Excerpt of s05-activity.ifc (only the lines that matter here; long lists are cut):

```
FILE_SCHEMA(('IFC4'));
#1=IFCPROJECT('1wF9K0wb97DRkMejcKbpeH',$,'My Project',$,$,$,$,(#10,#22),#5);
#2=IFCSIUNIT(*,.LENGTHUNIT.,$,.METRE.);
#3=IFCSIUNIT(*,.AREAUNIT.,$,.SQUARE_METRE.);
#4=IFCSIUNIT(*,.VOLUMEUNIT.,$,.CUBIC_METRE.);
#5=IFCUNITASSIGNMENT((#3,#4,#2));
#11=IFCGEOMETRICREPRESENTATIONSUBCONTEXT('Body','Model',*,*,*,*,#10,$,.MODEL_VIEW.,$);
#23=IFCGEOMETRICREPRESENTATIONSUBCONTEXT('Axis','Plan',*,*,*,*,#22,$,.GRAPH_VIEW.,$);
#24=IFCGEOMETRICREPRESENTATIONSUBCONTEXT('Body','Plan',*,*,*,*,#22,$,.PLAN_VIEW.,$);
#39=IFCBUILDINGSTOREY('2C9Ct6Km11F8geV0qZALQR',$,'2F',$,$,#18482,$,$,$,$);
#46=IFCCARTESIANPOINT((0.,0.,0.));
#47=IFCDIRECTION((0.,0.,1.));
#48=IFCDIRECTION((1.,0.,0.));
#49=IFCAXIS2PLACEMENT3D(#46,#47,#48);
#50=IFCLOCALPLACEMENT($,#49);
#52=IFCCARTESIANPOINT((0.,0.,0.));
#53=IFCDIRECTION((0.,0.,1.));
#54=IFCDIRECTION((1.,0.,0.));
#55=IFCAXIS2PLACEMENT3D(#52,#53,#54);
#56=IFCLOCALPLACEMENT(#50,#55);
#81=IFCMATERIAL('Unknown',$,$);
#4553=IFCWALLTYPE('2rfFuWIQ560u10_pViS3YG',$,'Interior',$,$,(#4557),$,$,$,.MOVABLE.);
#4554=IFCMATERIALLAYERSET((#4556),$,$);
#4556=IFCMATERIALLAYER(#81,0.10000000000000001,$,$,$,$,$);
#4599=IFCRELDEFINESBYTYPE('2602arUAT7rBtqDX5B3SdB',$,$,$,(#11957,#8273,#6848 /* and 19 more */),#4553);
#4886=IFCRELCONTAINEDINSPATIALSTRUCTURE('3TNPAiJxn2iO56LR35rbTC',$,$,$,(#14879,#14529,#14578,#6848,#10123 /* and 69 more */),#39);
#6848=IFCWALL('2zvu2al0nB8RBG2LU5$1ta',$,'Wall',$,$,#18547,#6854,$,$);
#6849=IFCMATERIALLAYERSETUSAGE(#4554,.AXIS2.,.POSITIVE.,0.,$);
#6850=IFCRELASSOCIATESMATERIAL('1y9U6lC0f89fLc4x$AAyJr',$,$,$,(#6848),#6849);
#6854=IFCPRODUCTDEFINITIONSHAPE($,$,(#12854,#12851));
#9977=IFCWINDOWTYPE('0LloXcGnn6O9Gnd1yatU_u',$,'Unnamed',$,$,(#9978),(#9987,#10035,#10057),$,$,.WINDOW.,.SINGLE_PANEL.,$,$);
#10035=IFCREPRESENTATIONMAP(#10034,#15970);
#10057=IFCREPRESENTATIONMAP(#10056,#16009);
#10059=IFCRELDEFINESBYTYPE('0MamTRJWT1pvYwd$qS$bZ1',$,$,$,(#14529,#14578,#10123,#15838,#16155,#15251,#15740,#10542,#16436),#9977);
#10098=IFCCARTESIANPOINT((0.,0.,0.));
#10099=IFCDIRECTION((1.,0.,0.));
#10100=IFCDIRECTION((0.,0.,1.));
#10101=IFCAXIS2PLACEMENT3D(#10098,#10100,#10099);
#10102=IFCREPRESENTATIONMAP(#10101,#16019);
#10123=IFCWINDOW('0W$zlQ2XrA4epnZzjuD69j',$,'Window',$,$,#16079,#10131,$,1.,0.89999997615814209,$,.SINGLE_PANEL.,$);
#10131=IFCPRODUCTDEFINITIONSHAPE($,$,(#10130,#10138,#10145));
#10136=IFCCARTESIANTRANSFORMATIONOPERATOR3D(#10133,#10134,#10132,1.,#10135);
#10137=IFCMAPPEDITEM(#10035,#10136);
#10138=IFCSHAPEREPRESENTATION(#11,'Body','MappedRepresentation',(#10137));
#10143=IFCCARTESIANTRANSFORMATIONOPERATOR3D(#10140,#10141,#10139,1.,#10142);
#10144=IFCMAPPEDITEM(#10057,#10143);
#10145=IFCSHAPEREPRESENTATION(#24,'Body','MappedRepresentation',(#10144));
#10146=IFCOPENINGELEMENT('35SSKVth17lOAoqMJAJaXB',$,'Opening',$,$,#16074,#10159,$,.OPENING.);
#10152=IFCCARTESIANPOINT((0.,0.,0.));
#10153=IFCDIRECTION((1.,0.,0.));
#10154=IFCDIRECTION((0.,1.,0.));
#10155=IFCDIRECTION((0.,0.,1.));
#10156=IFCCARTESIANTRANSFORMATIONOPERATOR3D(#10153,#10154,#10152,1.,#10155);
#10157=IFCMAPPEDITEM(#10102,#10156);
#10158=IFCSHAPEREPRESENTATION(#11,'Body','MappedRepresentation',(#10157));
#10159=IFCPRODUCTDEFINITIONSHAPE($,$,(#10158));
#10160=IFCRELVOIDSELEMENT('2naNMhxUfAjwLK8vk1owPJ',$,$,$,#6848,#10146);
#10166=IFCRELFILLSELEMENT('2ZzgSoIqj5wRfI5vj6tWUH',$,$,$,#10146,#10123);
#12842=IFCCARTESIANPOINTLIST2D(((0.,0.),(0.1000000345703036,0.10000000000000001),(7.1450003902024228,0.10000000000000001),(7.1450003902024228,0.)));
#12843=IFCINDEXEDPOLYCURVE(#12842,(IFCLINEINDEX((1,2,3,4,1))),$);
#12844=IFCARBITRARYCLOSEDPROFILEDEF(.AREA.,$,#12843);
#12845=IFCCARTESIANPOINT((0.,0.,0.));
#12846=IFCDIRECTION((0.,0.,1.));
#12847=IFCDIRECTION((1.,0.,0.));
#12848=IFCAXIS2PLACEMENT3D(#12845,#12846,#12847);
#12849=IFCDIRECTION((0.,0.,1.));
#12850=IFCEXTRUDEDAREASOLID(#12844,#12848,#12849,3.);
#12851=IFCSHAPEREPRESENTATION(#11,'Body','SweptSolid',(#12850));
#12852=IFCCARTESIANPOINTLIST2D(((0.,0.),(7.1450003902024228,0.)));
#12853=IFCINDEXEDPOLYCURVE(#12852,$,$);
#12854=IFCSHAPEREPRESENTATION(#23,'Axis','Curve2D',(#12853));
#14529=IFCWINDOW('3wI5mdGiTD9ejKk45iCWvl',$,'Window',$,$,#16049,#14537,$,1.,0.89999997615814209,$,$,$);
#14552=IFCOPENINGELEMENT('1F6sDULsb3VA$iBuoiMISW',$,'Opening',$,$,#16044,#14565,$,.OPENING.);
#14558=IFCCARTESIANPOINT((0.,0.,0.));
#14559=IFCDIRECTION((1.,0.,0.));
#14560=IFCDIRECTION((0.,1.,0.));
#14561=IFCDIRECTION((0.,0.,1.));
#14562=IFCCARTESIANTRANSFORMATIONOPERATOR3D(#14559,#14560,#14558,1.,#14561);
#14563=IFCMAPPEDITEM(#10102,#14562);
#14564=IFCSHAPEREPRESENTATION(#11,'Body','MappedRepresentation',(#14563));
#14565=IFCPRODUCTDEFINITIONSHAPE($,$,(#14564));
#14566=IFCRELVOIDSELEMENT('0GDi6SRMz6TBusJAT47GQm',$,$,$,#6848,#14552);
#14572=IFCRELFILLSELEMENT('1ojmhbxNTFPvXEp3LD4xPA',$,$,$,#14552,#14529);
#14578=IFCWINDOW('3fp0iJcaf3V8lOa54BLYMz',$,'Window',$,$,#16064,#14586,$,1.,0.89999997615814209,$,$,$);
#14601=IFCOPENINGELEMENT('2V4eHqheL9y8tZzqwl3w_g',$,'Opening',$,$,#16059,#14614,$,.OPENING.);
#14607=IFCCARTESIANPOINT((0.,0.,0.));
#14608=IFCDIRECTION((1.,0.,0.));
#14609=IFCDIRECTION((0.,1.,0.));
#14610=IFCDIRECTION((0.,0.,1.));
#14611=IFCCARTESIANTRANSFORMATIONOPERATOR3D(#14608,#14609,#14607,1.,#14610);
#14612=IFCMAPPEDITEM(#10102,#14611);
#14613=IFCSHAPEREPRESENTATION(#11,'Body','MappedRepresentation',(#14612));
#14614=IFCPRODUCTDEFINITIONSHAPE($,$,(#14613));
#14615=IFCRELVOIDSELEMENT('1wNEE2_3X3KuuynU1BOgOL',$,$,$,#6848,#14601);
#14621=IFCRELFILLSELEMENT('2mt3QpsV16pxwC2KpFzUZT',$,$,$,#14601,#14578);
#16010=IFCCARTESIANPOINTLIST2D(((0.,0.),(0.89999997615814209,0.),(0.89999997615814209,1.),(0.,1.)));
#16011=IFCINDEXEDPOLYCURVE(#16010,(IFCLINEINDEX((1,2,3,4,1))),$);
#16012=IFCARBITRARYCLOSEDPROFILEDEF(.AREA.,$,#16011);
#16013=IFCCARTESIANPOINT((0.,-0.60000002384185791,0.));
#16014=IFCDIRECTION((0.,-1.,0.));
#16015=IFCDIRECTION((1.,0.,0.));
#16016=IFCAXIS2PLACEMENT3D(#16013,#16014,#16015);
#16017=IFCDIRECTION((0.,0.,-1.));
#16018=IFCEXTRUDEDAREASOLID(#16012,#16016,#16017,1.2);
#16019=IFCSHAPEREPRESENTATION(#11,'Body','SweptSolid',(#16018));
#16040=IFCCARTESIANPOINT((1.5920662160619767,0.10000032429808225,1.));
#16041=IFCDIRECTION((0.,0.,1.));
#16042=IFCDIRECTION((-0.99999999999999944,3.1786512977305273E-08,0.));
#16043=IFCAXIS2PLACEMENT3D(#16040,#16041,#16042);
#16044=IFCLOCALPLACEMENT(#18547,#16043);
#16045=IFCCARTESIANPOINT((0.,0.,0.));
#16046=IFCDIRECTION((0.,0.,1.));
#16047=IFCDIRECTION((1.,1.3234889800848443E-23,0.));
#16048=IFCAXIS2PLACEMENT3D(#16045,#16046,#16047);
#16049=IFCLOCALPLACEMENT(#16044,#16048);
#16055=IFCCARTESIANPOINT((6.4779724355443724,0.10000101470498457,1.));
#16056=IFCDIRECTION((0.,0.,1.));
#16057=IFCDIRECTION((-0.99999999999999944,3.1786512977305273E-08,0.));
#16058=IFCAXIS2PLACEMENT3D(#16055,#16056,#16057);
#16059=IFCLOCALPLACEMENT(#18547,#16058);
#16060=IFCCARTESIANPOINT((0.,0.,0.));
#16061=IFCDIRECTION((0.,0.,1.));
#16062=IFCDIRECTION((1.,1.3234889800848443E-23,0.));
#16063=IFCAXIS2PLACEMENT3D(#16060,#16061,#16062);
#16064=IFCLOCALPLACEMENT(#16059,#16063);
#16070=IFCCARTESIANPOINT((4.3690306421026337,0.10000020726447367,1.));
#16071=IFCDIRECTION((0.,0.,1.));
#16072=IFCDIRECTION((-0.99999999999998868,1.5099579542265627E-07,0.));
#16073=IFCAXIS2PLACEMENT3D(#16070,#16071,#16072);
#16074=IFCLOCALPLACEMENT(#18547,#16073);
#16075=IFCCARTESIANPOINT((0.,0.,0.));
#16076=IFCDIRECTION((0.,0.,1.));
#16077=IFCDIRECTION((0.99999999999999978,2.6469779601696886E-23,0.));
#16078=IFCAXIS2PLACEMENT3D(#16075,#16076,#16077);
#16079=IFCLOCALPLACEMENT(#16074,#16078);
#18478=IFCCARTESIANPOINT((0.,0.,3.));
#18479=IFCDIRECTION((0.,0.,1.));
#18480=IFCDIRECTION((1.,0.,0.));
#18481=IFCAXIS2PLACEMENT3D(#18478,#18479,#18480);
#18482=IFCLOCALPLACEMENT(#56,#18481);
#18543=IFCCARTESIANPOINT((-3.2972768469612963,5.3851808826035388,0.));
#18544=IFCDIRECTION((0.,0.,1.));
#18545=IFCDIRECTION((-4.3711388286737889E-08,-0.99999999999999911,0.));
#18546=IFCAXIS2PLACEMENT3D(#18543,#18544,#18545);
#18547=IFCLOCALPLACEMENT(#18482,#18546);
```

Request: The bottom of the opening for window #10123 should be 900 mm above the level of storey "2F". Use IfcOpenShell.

```python
import numpy as np
import ifcopenshell
import ifcopenshell.api.geometry
import ifcopenshell.geom
import ifcopenshell.util.element
import ifcopenshell.util.placement
import ifcopenshell.util.shape
import ifcopenshell.util.unit

model = ifcopenshell.open("s05-activity.ifc")
unit_scale = ifcopenshell.util.unit.calculate_unit_scale(model)

window = model.by_guid("0W$zlQ2XrA4epnZzjuD69j")
opening = window.FillsVoids[0].RelatingOpeningElement
storey = ifcopenshell.util.element.get_container(window, ifc_class="IfcBuildingStorey")
level = ifcopenshell.util.placement.get_local_placement(storey.ObjectPlacement)[2, 3]

# The opening's origin need not be at the sill, so measure its lowest point.
shape = ifcopenshell.geom.create_shape(ifcopenshell.geom.settings(), opening)
bottom = ifcopenshell.util.shape.get_shape_bottom_elevation(shape, shape.geometry) / unit_scale
dz = level + 0.9 - bottom

shift = np.array([0.0, 0.0, dz])
# The window is placed relative to its opening, so it follows when the opening moves.
matrix = ifcopenshell.util.placement.get_local_placement(opening.ObjectPlacement)
matrix[:3, 3] += shift
ifcopenshell.api.geometry.edit_object_placement(
    model, product=opening, matrix=matrix, is_si=False, should_transform_children=True
)

print(f"moved by {dz * unit_scale:+.3f} m")

model.write("s05-activity_rev.ifc")
```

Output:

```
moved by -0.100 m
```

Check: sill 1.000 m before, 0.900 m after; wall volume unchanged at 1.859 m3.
